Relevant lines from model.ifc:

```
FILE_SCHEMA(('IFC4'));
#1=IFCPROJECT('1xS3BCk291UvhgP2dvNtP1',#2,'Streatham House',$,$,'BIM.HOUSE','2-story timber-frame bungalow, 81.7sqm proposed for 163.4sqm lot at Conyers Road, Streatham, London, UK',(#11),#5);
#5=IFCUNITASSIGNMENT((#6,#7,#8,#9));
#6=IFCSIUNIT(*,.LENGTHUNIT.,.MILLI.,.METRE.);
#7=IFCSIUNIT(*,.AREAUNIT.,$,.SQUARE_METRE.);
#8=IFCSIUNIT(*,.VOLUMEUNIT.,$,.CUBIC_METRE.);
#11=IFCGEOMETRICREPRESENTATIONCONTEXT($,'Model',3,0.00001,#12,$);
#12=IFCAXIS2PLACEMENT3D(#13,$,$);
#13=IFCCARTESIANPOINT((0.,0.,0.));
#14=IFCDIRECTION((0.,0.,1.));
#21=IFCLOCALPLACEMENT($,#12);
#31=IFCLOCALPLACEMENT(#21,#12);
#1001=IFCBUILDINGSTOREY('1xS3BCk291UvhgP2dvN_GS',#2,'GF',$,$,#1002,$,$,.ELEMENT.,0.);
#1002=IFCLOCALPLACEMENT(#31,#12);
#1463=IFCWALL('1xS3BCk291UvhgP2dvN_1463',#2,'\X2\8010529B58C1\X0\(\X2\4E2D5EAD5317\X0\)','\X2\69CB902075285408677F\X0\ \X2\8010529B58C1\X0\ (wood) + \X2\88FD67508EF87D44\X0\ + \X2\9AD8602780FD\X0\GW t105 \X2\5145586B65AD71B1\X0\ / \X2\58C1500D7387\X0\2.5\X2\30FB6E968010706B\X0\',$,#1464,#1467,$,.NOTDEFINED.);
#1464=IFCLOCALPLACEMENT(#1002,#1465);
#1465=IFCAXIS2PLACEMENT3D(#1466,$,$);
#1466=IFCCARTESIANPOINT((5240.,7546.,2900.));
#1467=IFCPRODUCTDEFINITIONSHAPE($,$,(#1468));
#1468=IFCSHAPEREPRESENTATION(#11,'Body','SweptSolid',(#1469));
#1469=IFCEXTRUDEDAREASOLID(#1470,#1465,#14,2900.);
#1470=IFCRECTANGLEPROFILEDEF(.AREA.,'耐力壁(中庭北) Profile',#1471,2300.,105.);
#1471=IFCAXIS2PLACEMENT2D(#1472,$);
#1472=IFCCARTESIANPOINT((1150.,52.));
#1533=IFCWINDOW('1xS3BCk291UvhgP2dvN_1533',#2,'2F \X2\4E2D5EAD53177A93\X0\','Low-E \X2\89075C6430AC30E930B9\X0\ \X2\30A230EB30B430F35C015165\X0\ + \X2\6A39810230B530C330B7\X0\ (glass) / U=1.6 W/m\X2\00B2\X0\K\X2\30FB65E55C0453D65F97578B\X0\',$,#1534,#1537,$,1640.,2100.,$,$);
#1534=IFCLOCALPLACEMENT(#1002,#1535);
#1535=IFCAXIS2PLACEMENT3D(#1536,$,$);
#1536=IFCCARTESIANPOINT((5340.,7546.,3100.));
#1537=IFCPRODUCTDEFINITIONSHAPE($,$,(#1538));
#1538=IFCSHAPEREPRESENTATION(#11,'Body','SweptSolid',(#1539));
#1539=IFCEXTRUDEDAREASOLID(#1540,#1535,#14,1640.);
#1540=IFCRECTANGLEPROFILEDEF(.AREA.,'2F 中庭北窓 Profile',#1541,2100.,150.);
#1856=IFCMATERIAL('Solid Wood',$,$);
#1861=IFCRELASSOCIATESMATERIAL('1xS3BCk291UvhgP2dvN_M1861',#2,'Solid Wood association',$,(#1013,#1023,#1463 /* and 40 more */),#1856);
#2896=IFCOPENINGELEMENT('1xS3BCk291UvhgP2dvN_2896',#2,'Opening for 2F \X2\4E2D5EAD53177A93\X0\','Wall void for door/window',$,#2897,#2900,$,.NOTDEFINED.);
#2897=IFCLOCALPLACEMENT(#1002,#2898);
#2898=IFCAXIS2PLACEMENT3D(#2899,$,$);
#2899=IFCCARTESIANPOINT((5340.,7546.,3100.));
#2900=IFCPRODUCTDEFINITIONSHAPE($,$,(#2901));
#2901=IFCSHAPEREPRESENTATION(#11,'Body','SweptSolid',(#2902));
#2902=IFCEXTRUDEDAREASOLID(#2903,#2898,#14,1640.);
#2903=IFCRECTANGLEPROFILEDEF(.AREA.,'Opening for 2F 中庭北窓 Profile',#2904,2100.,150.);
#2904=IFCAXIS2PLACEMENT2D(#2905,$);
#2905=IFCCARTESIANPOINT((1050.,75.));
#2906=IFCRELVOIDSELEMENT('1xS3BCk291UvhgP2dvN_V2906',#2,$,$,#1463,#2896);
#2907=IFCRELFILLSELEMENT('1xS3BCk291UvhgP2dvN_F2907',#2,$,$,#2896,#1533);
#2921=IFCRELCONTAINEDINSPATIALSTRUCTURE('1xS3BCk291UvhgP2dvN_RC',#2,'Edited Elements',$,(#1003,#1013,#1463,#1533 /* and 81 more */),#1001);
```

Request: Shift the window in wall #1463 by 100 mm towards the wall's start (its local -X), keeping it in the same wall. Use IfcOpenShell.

```python
import ifcopenshell
import ifcopenshell.api.geometry
import ifcopenshell.util.placement

model = ifcopenshell.open("model.ifc")

window = model.by_guid("1xS3BCk291UvhgP2dvN_1533")
opening = window.FillsVoids[0].RelatingOpeningElement
wall = opening.VoidsElements[0].RelatingBuildingElement

wall_matrix = ifcopenshell.util.placement.get_local_placement(wall.ObjectPlacement)
shift = wall_matrix[:3, 0] * -100.0
before = ifcopenshell.util.placement.get_local_placement(window.ObjectPlacement)[:3, 3].copy()

# The window is not placed relative to its opening, so move both.
for product in (opening, window):
    matrix = ifcopenshell.util.placement.get_local_placement(product.ObjectPlacement)
    matrix[:3, 3] += shift
    ifcopenshell.api.geometry.edit_object_placement(model, product=product, matrix=matrix, is_si=False)

after = ifcopenshell.util.placement.get_local_placement(window.ObjectPlacement)[:3, 3]
print("window moved by", (after - before).round(3) + 0.0)

model.write("model_updated.ifc")
```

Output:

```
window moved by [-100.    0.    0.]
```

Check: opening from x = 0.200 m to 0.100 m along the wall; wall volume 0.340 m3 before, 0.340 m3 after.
